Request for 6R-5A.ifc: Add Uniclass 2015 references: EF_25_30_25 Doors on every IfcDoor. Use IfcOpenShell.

First a look at what the model holds.

```python
import ifcopenshell

model = ifcopenshell.open("6R-5A.ifc")
print(model.schema)
print("classifications:", [c.Name for c in model.by_type("IfcClassification")])
for ifc_class in ("IfcDoor", "IfcRoof", "IfcStair", "IfcWall", "IfcWindow"):
    print(ifc_class, len(model.by_type(ifc_class)))
```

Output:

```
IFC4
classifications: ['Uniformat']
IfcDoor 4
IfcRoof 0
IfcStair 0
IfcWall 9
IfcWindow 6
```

```python
import ifcopenshell
import ifcopenshell.api.classification

model = ifcopenshell.open("6R-5A.ifc")

system = ifcopenshell.api.classification.add_classification(model, classification="Uniclass 2015")

codes = {
    "IfcDoor": ("EF_25_30_25", "Doors"),
}
for ifc_class, (code, name) in codes.items():
    products = model.by_type(ifc_class)
    ifcopenshell.api.classification.add_reference(
        model, products=products, classification=system, identification=code, name=name
    )
    print(code, len(products))

model.write("6R-5A_updated.ifc")
```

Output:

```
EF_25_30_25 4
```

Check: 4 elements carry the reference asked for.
